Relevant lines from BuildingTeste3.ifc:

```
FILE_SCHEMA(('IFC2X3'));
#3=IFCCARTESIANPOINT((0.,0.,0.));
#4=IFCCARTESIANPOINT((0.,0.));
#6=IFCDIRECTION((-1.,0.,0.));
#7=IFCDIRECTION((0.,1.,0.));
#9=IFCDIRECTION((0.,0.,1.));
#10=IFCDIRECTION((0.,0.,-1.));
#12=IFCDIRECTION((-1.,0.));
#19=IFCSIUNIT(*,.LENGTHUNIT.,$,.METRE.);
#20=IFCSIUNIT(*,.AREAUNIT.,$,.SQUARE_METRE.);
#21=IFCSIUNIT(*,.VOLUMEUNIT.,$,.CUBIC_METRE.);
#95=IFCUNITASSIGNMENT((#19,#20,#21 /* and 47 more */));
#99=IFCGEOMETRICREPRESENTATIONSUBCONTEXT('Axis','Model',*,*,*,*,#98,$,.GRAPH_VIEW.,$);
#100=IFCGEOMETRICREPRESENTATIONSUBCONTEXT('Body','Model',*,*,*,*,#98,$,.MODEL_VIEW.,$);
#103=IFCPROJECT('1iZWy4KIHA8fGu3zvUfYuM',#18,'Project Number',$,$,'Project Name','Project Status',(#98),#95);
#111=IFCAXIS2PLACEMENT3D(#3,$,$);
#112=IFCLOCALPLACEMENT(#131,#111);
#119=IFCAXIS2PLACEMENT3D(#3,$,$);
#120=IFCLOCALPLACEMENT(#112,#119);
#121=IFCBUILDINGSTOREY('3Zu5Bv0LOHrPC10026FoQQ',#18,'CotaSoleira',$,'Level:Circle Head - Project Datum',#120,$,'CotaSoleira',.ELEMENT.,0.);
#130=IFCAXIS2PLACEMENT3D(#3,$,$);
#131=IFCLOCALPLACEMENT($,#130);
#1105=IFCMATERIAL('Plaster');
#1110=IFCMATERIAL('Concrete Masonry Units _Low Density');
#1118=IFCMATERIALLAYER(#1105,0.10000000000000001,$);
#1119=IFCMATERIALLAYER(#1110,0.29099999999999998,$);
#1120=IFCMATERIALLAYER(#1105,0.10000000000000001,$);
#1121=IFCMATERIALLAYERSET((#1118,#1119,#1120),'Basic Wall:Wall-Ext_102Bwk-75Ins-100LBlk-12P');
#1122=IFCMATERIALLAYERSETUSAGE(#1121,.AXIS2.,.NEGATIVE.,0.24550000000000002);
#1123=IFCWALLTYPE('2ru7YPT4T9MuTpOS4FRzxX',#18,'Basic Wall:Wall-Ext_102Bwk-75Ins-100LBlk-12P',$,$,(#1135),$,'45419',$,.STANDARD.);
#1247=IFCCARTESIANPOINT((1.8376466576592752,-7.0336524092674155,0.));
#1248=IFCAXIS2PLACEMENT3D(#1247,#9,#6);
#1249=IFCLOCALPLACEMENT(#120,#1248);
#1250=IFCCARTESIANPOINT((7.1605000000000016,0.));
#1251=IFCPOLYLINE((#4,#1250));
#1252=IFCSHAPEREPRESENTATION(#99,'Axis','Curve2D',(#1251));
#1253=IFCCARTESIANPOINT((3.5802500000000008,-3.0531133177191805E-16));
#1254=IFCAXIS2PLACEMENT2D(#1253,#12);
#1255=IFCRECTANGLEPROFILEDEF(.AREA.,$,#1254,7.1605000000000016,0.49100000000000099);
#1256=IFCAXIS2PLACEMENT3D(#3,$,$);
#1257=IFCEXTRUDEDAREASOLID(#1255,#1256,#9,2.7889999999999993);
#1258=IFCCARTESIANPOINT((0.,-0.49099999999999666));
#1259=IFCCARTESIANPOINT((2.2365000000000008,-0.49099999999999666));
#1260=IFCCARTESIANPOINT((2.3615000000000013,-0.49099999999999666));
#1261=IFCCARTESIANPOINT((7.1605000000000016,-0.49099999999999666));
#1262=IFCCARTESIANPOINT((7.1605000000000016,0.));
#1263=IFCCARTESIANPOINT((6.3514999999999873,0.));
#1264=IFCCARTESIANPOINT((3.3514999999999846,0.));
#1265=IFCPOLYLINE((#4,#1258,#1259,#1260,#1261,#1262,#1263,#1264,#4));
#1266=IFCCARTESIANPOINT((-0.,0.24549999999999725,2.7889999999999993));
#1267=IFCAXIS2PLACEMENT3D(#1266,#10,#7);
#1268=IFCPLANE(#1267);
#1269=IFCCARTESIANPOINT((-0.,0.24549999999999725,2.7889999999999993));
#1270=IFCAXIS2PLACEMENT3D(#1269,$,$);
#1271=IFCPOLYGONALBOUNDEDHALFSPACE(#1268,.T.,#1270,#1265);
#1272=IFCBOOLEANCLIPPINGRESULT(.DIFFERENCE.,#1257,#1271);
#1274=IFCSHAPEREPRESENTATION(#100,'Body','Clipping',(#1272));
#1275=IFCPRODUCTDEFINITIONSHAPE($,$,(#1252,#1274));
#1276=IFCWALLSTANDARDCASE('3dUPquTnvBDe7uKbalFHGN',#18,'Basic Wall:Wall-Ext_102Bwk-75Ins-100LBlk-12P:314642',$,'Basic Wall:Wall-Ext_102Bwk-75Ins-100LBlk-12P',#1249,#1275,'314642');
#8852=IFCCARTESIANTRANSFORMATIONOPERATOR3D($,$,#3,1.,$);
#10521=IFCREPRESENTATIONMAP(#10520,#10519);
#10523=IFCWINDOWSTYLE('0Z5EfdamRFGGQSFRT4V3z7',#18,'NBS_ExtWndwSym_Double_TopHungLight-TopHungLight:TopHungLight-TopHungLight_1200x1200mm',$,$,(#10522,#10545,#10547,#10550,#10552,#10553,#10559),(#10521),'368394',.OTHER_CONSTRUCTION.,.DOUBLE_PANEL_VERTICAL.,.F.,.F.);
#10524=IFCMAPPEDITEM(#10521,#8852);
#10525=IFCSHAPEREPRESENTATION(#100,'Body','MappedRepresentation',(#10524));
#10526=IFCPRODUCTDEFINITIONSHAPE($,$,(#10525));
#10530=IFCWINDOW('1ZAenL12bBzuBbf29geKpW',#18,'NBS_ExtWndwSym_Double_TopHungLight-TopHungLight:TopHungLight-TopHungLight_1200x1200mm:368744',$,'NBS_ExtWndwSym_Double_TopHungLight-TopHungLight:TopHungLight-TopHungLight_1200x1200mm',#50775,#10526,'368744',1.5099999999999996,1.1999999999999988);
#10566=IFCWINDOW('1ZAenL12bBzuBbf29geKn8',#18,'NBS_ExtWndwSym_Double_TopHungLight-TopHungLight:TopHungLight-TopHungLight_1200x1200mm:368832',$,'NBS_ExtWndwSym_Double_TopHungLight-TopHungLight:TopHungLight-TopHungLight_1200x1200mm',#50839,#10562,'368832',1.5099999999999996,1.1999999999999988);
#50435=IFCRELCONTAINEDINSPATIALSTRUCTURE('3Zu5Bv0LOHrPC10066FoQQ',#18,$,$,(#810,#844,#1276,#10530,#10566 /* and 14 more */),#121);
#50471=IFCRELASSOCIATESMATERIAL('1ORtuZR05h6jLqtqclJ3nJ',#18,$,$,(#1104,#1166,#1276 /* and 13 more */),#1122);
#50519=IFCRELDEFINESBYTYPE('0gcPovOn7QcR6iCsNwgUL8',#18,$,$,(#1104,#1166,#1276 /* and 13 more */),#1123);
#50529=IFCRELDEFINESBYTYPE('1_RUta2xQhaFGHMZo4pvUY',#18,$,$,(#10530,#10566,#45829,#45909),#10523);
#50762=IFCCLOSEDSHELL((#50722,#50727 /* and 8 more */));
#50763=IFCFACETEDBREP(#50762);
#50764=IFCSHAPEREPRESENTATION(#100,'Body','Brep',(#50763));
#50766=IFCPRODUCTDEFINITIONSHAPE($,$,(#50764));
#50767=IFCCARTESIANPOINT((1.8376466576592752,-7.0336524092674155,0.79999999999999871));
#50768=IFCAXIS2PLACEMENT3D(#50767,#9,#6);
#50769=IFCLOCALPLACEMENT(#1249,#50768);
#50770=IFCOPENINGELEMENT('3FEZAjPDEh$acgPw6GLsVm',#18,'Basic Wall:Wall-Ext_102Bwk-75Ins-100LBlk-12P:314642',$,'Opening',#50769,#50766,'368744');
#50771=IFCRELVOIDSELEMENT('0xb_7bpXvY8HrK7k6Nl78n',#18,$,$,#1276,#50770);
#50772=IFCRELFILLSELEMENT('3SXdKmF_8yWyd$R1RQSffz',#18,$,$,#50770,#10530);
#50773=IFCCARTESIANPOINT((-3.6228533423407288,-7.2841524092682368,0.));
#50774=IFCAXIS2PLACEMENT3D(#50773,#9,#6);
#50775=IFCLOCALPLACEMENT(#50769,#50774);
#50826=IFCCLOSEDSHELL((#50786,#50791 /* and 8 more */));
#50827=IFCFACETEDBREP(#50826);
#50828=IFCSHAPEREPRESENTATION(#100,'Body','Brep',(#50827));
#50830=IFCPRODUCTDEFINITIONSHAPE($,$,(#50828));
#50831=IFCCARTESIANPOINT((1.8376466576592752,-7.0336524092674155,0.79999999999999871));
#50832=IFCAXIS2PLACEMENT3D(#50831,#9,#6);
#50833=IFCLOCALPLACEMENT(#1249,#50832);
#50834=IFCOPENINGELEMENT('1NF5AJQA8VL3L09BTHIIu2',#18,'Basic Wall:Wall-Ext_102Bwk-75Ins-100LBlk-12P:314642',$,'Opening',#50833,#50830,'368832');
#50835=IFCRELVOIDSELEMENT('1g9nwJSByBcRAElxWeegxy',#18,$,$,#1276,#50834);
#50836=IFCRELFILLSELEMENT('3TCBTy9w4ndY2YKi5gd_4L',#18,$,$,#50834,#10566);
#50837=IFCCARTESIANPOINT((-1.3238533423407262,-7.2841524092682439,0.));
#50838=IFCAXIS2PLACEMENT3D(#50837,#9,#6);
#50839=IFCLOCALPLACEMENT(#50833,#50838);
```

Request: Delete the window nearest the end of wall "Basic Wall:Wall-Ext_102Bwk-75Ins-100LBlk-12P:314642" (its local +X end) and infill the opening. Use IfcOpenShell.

```python
import ifcopenshell
import ifcopenshell.api.feature
import ifcopenshell.api.root
import ifcopenshell.geom
import ifcopenshell.util.shape

model = ifcopenshell.open("BuildingTeste3.ifc")
settings = ifcopenshell.geom.settings()


def volume(element):
    """Net volume in cubic metres, openings subtracted."""
    shape = ifcopenshell.geom.create_shape(settings, element)
    return ifcopenshell.util.shape.get_volume(shape.geometry)


window = model.by_guid("1ZAenL12bBzuBbf29geKpW")
opening = window.FillsVoids[0].RelatingOpeningElement
wall = opening.VoidsElements[0].RelatingBuildingElement
before = volume(wall)

ifcopenshell.api.root.remove_product(model, product=window)
ifcopenshell.api.feature.remove_feature(model, feature=opening)

after = volume(wall)

print(f"wall volume {before:.3f} -> {after:.3f} m3")

model.write("BuildingTeste3_edited.ifc")
```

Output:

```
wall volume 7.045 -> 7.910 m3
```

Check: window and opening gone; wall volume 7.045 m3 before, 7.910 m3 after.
